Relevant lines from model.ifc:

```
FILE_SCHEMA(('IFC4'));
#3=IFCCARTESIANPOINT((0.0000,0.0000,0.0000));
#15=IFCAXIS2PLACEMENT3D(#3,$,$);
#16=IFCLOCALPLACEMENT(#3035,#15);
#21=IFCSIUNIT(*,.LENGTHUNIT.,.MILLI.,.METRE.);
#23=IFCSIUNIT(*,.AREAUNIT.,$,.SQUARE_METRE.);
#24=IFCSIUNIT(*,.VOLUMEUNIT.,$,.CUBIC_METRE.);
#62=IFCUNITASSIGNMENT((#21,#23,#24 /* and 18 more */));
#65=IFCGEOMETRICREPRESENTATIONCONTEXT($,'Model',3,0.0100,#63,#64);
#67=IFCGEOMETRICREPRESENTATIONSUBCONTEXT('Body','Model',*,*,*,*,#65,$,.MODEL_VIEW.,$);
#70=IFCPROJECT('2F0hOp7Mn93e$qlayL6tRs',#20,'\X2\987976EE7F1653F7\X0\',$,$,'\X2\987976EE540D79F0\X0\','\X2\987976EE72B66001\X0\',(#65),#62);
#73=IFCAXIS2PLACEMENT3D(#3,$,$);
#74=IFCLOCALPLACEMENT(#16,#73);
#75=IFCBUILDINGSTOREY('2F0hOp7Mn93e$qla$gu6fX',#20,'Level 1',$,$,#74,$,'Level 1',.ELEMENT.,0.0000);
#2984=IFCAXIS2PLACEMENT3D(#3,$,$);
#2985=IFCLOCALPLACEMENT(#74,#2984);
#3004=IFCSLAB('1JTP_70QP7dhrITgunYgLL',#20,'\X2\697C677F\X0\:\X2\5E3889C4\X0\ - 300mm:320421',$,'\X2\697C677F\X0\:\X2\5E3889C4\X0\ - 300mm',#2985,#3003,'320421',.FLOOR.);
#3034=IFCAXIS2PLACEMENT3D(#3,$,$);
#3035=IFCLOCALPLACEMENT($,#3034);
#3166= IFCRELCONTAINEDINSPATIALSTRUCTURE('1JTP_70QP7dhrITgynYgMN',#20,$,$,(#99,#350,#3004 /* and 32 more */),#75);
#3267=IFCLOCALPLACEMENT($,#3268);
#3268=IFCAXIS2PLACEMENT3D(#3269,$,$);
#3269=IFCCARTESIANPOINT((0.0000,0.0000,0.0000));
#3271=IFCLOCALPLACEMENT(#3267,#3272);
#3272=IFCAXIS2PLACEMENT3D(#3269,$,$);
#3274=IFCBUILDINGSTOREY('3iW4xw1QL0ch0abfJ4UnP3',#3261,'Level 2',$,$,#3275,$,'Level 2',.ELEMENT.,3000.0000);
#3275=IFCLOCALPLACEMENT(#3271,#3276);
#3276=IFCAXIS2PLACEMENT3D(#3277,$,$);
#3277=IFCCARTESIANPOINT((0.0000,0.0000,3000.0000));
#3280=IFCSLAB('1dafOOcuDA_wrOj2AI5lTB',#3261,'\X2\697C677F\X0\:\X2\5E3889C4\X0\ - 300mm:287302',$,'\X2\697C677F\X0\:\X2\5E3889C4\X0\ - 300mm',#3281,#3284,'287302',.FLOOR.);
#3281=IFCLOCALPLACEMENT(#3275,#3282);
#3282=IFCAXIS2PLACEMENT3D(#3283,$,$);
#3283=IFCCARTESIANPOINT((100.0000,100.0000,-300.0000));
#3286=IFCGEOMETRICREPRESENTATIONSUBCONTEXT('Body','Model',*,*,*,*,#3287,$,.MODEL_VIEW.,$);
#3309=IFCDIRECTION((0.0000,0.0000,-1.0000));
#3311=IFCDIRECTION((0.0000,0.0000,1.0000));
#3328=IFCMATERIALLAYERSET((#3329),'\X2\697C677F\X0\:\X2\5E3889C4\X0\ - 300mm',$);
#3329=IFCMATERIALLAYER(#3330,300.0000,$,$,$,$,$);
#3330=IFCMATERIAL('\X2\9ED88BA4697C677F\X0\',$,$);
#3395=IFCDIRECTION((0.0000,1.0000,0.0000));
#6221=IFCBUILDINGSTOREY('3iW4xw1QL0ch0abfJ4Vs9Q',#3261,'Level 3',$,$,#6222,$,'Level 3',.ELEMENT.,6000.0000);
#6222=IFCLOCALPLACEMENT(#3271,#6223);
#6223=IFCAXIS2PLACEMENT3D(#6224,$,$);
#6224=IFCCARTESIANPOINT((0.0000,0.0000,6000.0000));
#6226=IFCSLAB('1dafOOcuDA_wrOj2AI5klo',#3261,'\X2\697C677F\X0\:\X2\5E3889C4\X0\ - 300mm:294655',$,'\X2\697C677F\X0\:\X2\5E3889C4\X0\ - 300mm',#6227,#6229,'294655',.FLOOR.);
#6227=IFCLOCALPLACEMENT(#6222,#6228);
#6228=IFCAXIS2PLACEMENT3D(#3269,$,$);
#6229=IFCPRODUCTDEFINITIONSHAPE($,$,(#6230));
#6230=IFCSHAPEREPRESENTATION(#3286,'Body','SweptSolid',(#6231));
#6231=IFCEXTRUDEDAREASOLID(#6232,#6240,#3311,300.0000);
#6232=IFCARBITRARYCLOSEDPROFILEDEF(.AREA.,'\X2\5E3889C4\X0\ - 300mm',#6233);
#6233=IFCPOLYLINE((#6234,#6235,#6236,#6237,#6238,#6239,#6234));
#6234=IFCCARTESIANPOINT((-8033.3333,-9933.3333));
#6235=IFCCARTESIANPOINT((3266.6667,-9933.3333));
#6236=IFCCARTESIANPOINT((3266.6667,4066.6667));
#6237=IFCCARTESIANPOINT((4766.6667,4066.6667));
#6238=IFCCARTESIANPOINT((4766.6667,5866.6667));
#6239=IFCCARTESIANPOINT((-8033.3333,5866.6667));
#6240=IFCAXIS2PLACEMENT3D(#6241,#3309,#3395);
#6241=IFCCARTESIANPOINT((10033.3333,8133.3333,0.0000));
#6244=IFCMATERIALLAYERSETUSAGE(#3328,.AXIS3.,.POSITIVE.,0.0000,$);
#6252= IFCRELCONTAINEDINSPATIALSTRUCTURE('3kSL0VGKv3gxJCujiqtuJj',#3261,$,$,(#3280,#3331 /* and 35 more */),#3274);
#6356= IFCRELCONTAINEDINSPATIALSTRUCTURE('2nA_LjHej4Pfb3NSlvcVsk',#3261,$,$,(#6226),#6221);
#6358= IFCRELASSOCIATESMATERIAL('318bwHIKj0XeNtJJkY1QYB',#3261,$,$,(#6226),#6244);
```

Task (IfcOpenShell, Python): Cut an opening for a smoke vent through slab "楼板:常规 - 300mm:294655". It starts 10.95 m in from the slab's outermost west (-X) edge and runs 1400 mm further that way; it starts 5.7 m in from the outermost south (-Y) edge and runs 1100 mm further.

```python
import numpy as np
import ifcopenshell
import ifcopenshell.api.feature
import ifcopenshell.api.geometry
import ifcopenshell.api.root
import ifcopenshell.geom
import ifcopenshell.util.placement
import ifcopenshell.util.representation
import ifcopenshell.util.shape
import ifcopenshell.util.unit

model = ifcopenshell.open("model.ifc")
unit_scale = ifcopenshell.util.unit.calculate_unit_scale(model)
settings = ifcopenshell.geom.settings()


def volume(element):
    """Net volume in cubic metres, openings subtracted."""
    shape = ifcopenshell.geom.create_shape(settings, element)
    return ifcopenshell.util.shape.get_volume(shape.geometry)


slab = model.by_guid("1dafOOcuDA_wrOj2AI5klo")
before = volume(slab)

# Extent in the slab's own axes, in metres. The edges named are its -X and -Y sides.
slab_shape = ifcopenshell.geom.create_shape(settings, slab)
vertices = ifcopenshell.util.shape.get_vertices(slab_shape.geometry)
x_min, y_min, bottom = vertices.min(axis=0)
top = vertices[:, 2].max()

opening = ifcopenshell.api.root.create_entity(model, ifc_class="IfcOpeningElement", name="Smoke vent opening", predefined_type="OPENING")
context = ifcopenshell.util.representation.get_context(model, "Model", "Body", "MODEL_VIEW")
width, depth = 1.4, 1.1
outline = [(0.0, 0.0), (width, 0.0), (width, depth), (0.0, depth), (0.0, 0.0)]
# Overshoot both faces by 50 mm so the cut is clean.
shape = ifcopenshell.api.geometry.add_slab_representation(
    model, context=context, depth=top - bottom + 0.1, polyline=outline
)
ifcopenshell.api.geometry.assign_representation(model, product=opening, representation=shape)

matrix = ifcopenshell.util.placement.get_local_placement(slab.ObjectPlacement)
matrix[:, 3] = matrix @ np.append(np.array([x_min + 10.95, y_min + 5.7, bottom - 0.05]) / unit_scale, 1.0)
ifcopenshell.api.geometry.edit_object_placement(model, product=opening, matrix=matrix, is_si=False)
ifcopenshell.api.feature.add_feature(model, feature=opening, element=slab)

after = volume(slab)

print(f"slab volume {before:.3f} -> {after:.3f} m3")

model.write("model_v2.ifc")
```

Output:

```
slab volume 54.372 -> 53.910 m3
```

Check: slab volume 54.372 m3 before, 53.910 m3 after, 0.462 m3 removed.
